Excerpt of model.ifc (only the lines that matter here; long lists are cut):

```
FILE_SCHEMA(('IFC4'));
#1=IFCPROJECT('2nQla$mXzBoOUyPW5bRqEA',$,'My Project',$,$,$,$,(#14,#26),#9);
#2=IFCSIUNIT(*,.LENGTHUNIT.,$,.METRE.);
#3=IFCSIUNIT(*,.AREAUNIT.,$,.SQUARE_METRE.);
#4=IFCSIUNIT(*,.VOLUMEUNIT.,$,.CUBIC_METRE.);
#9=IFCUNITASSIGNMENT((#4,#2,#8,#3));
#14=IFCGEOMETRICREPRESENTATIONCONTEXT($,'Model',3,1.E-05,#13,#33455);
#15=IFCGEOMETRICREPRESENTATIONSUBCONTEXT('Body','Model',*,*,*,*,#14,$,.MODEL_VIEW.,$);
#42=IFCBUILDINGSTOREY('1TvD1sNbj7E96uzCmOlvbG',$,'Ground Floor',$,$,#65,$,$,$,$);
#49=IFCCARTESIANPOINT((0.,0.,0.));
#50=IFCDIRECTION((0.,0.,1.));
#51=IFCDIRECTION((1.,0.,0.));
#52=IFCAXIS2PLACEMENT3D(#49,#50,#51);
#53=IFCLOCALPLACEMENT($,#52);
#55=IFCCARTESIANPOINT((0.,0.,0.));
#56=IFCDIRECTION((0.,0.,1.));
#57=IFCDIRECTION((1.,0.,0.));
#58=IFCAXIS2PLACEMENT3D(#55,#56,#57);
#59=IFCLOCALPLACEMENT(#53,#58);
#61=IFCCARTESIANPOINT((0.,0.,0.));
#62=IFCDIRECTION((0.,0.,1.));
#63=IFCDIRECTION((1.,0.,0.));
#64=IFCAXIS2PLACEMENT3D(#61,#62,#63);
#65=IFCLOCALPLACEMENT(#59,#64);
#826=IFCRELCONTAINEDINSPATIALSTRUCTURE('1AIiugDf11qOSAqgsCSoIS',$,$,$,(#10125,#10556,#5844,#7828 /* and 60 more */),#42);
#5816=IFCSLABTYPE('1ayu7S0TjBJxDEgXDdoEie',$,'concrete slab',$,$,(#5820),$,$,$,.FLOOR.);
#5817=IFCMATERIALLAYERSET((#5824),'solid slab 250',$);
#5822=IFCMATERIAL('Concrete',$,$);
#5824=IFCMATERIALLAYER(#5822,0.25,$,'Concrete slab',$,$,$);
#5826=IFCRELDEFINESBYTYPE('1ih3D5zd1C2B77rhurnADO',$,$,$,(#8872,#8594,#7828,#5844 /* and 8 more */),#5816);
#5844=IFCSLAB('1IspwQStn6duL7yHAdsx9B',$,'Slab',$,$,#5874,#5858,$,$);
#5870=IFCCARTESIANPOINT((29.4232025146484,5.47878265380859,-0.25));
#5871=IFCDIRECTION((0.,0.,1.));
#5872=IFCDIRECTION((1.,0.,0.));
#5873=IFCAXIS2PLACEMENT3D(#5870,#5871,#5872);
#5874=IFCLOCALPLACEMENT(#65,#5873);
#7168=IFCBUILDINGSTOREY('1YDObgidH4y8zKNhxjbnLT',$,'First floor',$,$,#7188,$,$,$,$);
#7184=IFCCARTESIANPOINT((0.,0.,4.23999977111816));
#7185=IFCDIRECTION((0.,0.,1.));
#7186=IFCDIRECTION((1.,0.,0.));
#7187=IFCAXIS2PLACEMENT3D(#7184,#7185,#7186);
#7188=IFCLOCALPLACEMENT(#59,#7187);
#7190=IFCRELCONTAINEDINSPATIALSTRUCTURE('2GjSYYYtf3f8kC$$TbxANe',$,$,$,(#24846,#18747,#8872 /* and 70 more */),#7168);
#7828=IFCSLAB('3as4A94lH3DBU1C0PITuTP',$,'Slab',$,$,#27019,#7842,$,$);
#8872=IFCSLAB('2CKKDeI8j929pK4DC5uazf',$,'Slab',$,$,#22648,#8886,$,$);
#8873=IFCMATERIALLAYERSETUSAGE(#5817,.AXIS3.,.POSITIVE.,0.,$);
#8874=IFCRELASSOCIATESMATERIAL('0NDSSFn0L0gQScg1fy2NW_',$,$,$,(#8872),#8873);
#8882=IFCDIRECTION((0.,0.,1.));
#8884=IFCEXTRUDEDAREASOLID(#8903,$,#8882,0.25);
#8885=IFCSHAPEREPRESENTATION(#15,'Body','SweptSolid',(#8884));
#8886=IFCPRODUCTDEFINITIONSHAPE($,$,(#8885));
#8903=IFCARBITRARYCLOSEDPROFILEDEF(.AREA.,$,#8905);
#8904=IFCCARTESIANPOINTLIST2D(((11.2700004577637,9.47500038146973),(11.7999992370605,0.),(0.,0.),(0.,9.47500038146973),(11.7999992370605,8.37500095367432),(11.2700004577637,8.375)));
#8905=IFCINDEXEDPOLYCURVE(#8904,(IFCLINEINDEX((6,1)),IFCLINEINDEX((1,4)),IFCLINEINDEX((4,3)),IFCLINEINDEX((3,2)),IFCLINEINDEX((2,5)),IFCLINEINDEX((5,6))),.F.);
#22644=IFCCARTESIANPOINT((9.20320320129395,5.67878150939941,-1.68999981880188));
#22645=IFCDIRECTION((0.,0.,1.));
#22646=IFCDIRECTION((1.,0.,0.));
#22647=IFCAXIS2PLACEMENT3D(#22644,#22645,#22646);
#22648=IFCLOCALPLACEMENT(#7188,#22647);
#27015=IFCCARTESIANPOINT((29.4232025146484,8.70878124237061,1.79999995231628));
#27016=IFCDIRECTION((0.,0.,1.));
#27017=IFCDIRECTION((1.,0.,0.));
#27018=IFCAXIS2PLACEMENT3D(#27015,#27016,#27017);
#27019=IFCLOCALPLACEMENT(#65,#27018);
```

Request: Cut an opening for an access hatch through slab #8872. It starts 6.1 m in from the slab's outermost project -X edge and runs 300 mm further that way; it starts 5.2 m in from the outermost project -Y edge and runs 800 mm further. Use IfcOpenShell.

```python
import numpy as np
import ifcopenshell
import ifcopenshell.api.feature
import ifcopenshell.api.geometry
import ifcopenshell.api.root
import ifcopenshell.geom
import ifcopenshell.util.placement
import ifcopenshell.util.representation
import ifcopenshell.util.shape
import ifcopenshell.util.unit

model = ifcopenshell.open("model.ifc")
unit_scale = ifcopenshell.util.unit.calculate_unit_scale(model)
settings = ifcopenshell.geom.settings()


def volume(element):
    """Net volume in cubic metres, openings subtracted."""
    shape = ifcopenshell.geom.create_shape(settings, element)
    return ifcopenshell.util.shape.get_volume(shape.geometry)


slab = model.by_guid("2CKKDeI8j929pK4DC5uazf")
before = volume(slab)

# Extent in the slab's own axes, in metres. The edges named are its -X and -Y sides.
slab_shape = ifcopenshell.geom.create_shape(settings, slab)
vertices = ifcopenshell.util.shape.get_vertices(slab_shape.geometry)
x_min, y_min, bottom = vertices.min(axis=0)
top = vertices[:, 2].max()

opening = ifcopenshell.api.root.create_entity(model, ifc_class="IfcOpeningElement", name="Access hatch opening", predefined_type="OPENING")
context = ifcopenshell.util.representation.get_context(model, "Model", "Body", "MODEL_VIEW")
width, depth = 0.3, 0.8
outline = [(0.0, 0.0), (width, 0.0), (width, depth), (0.0, depth), (0.0, 0.0)]
# Overshoot both faces by 50 mm so the cut is clean.
shape = ifcopenshell.api.geometry.add_slab_representation(
    model, context=context, depth=top - bottom + 0.1, polyline=outline
)
ifcopenshell.api.geometry.assign_representation(model, product=opening, representation=shape)

matrix = ifcopenshell.util.placement.get_local_placement(slab.ObjectPlacement)
matrix[:, 3] = matrix @ np.append(np.array([x_min + 6.1, y_min + 5.2, bottom - 0.05]) / unit_scale, 1.0)
ifcopenshell.api.geometry.edit_object_placement(model, product=opening, matrix=matrix, is_si=False)
ifcopenshell.api.feature.add_feature(model, feature=opening, element=slab)

after = volume(slab)

print(f"slab volume {before:.3f} -> {after:.3f} m3")

model.write("model-out.ifc")
```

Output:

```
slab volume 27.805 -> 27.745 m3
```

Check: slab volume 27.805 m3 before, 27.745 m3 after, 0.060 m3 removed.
